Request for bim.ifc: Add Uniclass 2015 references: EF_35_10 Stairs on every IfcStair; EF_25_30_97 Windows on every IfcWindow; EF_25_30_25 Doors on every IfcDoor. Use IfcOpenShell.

First a look at what the model holds.

```python
import ifcopenshell

model = ifcopenshell.open("bim.ifc")
print(model.schema)
print("classifications:", [c.Name for c in model.by_type("IfcClassification")])
for ifc_class in ("IfcDoor", "IfcRoof", "IfcStair", "IfcWall", "IfcWindow"):
    print(ifc_class, len(model.by_type(ifc_class)))
```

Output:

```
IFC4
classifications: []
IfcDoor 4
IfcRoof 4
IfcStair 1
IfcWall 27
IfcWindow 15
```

```python
import ifcopenshell
import ifcopenshell.api.classification

model = ifcopenshell.open("bim.ifc")

system = ifcopenshell.api.classification.add_classification(model, classification="Uniclass 2015")

codes = {
    "IfcStair": ("EF_35_10", "Stairs"),
    "IfcWindow": ("EF_25_30_97", "Windows"),
    "IfcDoor": ("EF_25_30_25", "Doors"),
}
for ifc_class, (code, name) in codes.items():
    products = model.by_type(ifc_class)
    ifcopenshell.api.classification.add_reference(
        model, products=products, classification=system, identification=code, name=name
    )
    print(code, len(products))

model.write("bim_edited.ifc")
```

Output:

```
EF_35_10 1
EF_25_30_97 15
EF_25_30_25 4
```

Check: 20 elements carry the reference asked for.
